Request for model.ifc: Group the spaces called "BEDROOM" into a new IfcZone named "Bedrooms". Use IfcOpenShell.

First a look at what the model holds.

```python
import ifcopenshell

model = ifcopenshell.open("model.ifc")
print(model.schema)
seen = {}
for space in model.by_type("IfcSpace"):
    seen[space.LongName] = seen.get(space.LongName, 0) + 1
for name, count in sorted(seen.items(), key=str):
    print(count, "x", name)
print("zones:", [z.Name for z in model.by_type("IfcZone")][:20])
```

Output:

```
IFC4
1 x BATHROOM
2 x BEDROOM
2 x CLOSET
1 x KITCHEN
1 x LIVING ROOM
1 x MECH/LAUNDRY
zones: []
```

```python
import ifcopenshell
import ifcopenshell.api.group
import ifcopenshell.api.root

model = ifcopenshell.open("model.ifc")

names = {"BEDROOM"}
spaces = [s for s in model.by_type("IfcSpace") if s.LongName in names]

zone = ifcopenshell.api.root.create_entity(model, ifc_class="IfcZone", name="Bedrooms")
ifcopenshell.api.group.assign_group(model, products=spaces, group=zone)
print(len(spaces), "spaces in", zone.Name)

model.write("model_updated.ifc")
```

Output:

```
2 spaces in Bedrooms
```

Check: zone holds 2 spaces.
